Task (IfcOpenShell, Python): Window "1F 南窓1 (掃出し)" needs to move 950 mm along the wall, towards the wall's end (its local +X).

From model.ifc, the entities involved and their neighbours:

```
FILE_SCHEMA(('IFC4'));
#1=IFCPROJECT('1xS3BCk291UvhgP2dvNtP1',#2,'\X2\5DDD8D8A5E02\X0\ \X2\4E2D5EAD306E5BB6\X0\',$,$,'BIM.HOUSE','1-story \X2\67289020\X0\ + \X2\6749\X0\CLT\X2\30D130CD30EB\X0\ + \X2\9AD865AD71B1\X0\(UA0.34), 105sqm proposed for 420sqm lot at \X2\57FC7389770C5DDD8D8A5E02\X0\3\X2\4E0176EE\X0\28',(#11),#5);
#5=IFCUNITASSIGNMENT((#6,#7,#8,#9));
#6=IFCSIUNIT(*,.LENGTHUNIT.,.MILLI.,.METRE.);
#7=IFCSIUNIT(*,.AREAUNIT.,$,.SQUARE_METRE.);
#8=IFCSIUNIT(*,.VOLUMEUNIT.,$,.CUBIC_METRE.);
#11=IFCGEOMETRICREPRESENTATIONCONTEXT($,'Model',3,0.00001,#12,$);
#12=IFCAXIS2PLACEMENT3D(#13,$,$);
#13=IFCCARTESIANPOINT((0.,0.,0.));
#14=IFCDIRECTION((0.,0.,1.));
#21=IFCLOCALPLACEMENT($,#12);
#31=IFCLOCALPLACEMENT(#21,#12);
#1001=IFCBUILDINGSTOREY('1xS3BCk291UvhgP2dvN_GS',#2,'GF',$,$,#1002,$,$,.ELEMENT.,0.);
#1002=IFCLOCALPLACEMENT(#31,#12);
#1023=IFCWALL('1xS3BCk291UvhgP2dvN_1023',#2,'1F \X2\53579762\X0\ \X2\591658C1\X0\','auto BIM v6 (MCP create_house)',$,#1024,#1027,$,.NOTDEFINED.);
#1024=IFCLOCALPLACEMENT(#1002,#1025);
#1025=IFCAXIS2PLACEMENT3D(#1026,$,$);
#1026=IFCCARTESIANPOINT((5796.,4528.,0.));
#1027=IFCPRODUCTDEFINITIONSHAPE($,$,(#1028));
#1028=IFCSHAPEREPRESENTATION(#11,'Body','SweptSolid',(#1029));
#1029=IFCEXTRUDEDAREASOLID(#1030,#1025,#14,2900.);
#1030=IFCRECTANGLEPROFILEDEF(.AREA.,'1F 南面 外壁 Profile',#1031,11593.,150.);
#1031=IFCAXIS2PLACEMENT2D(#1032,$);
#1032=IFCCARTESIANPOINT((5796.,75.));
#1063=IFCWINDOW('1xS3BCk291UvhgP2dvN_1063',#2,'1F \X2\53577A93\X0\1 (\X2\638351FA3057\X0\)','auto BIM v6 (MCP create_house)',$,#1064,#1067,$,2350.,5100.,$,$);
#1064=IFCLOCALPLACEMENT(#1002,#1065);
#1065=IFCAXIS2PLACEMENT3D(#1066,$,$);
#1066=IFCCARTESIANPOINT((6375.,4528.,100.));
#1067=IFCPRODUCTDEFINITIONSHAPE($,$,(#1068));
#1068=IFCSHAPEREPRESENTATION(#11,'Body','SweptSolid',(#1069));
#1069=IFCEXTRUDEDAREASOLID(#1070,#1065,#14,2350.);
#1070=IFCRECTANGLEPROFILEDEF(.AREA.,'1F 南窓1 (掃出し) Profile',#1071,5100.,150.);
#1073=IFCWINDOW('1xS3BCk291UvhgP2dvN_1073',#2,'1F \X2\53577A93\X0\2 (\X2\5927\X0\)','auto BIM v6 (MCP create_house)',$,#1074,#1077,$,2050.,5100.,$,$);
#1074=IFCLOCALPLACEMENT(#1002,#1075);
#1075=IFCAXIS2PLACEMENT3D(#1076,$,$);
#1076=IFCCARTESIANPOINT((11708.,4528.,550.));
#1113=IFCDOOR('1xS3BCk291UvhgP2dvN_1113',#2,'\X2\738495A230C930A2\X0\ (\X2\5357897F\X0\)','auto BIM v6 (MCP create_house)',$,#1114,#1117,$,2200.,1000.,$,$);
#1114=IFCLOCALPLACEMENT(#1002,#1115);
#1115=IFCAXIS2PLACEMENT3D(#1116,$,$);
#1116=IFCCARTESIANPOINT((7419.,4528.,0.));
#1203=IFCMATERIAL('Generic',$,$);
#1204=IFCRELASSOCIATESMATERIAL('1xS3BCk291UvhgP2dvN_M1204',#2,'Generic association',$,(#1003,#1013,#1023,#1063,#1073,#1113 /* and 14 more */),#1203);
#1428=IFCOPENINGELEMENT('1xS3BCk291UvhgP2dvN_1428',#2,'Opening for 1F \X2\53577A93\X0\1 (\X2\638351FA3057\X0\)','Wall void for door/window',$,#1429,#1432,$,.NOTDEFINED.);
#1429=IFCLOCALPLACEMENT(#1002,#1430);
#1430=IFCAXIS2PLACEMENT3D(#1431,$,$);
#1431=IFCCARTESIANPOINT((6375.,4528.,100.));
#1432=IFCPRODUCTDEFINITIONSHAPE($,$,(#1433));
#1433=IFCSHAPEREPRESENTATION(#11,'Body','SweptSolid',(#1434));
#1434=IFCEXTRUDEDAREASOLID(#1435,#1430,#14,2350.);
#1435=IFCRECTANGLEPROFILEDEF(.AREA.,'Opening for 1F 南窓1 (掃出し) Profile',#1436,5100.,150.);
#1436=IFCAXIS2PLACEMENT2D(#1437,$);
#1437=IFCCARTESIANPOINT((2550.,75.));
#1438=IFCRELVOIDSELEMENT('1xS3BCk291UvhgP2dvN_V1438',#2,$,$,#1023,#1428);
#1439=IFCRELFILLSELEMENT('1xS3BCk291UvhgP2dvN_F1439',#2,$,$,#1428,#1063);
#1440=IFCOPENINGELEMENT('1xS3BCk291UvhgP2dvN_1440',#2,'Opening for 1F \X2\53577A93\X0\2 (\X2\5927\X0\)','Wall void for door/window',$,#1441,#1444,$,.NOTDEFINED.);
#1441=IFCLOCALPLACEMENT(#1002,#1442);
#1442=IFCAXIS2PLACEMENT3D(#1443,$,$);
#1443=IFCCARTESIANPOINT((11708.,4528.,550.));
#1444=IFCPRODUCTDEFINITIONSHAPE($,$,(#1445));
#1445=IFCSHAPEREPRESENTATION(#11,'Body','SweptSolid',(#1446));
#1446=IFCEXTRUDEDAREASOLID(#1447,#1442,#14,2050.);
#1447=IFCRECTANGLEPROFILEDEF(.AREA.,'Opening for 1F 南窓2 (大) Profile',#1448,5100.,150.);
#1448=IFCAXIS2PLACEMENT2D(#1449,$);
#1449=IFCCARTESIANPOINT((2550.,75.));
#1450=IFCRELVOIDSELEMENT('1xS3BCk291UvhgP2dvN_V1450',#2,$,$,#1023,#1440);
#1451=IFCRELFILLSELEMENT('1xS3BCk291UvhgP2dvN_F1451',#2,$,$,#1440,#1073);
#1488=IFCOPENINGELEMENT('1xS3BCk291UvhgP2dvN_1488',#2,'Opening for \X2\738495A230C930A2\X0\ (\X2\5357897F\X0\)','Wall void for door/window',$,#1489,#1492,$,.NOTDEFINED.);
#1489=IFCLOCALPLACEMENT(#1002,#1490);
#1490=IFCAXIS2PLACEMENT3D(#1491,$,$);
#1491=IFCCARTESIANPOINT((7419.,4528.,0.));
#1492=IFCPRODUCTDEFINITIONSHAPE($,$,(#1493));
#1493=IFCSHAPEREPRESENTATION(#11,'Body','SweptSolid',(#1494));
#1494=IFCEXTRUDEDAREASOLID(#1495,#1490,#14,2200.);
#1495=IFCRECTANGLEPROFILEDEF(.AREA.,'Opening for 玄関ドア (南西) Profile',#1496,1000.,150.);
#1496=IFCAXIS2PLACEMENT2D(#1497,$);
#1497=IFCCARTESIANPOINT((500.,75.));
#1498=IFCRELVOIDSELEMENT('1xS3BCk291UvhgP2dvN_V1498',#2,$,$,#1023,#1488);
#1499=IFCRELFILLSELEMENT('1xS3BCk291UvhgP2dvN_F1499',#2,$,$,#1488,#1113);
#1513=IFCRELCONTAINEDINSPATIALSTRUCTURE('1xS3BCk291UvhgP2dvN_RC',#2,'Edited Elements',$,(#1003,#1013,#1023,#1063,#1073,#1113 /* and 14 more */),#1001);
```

```python
import ifcopenshell
import ifcopenshell.api.geometry
import ifcopenshell.util.placement

model = ifcopenshell.open("model.ifc")

window = model.by_guid("1xS3BCk291UvhgP2dvN_1063")
opening = window.FillsVoids[0].RelatingOpeningElement
wall = opening.VoidsElements[0].RelatingBuildingElement

wall_matrix = ifcopenshell.util.placement.get_local_placement(wall.ObjectPlacement)
shift = wall_matrix[:3, 0] * 950.0
before = ifcopenshell.util.placement.get_local_placement(window.ObjectPlacement)[:3, 3].copy()

# The window is not placed relative to its opening, so move both.
for product in (opening, window):
    matrix = ifcopenshell.util.placement.get_local_placement(product.ObjectPlacement)
    matrix[:3, 3] += shift
    ifcopenshell.api.geometry.edit_object_placement(model, product=product, matrix=matrix, is_si=False)

after = ifcopenshell.util.placement.get_local_placement(window.ObjectPlacement)[:3, 3]
print("window moved by", (after - before).round(3) + 0.0)

model.write("model_v2.ifc")
```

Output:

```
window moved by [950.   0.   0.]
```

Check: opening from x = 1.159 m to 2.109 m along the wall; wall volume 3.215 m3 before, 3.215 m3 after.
